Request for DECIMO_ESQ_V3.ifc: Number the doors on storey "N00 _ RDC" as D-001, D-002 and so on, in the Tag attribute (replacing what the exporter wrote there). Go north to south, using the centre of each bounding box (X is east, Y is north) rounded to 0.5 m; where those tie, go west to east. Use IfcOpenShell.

First a look at what the model holds.

```python
import ifcopenshell
import ifcopenshell.util.element
import ifcopenshell.util.placement

model = ifcopenshell.open("DECIMO_ESQ_V3.ifc")
print(model.schema)
storey = next(s for s in model.by_type("IfcBuildingStorey") if s.Name == "N00 _ RDC")
doors = [e for e in ifcopenshell.util.element.get_decomposition(storey) if e.is_a("IfcDoor")]
for e in sorted(doors, key=lambda e: e.id()):
    origin = ifcopenshell.util.placement.get_local_placement(e.ObjectPlacement)[:3, 3]
    print(e.id(), e.Tag, e.Name, origin.round(2) + 0.0, sep=" | ")
```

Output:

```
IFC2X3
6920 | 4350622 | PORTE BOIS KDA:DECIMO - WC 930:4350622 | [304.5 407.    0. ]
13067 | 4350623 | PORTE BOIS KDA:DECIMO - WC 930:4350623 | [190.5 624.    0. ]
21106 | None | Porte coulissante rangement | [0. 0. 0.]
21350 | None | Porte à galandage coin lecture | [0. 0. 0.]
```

```python
import ifcopenshell
import ifcopenshell.geom
import ifcopenshell.util.element
import ifcopenshell.util.shape

model = ifcopenshell.open("DECIMO_ESQ_V3.ifc")
settings = ifcopenshell.geom.settings()
settings.set("use-world-coords", True)


def centre(element):
    shape = ifcopenshell.geom.create_shape(settings, element)
    return ifcopenshell.util.shape.get_bbox_centroid(shape.geometry)


storey = next(s for s in model.by_type("IfcBuildingStorey") if s.Name == "N00 _ RDC")
doors = [e for e in ifcopenshell.util.element.get_decomposition(storey) if e.is_a("IfcDoor")]

# Insertion points can sit at a corner or the storey origin, so sort by the geometry (in metres).
centres = {e: centre(e) for e in doors}
doors.sort(key=lambda e: (-round(centres[e][1] / 0.5), centres[e][0]))

for i, e in enumerate(doors, start=1):
    number = f"D-0{i:02d}"
    e.Tag = number
    print(e.id(), number)

model.write("DECIMO_ESQ_V3-out.ifc")
```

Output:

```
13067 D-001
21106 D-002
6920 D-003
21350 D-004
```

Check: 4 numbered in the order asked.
